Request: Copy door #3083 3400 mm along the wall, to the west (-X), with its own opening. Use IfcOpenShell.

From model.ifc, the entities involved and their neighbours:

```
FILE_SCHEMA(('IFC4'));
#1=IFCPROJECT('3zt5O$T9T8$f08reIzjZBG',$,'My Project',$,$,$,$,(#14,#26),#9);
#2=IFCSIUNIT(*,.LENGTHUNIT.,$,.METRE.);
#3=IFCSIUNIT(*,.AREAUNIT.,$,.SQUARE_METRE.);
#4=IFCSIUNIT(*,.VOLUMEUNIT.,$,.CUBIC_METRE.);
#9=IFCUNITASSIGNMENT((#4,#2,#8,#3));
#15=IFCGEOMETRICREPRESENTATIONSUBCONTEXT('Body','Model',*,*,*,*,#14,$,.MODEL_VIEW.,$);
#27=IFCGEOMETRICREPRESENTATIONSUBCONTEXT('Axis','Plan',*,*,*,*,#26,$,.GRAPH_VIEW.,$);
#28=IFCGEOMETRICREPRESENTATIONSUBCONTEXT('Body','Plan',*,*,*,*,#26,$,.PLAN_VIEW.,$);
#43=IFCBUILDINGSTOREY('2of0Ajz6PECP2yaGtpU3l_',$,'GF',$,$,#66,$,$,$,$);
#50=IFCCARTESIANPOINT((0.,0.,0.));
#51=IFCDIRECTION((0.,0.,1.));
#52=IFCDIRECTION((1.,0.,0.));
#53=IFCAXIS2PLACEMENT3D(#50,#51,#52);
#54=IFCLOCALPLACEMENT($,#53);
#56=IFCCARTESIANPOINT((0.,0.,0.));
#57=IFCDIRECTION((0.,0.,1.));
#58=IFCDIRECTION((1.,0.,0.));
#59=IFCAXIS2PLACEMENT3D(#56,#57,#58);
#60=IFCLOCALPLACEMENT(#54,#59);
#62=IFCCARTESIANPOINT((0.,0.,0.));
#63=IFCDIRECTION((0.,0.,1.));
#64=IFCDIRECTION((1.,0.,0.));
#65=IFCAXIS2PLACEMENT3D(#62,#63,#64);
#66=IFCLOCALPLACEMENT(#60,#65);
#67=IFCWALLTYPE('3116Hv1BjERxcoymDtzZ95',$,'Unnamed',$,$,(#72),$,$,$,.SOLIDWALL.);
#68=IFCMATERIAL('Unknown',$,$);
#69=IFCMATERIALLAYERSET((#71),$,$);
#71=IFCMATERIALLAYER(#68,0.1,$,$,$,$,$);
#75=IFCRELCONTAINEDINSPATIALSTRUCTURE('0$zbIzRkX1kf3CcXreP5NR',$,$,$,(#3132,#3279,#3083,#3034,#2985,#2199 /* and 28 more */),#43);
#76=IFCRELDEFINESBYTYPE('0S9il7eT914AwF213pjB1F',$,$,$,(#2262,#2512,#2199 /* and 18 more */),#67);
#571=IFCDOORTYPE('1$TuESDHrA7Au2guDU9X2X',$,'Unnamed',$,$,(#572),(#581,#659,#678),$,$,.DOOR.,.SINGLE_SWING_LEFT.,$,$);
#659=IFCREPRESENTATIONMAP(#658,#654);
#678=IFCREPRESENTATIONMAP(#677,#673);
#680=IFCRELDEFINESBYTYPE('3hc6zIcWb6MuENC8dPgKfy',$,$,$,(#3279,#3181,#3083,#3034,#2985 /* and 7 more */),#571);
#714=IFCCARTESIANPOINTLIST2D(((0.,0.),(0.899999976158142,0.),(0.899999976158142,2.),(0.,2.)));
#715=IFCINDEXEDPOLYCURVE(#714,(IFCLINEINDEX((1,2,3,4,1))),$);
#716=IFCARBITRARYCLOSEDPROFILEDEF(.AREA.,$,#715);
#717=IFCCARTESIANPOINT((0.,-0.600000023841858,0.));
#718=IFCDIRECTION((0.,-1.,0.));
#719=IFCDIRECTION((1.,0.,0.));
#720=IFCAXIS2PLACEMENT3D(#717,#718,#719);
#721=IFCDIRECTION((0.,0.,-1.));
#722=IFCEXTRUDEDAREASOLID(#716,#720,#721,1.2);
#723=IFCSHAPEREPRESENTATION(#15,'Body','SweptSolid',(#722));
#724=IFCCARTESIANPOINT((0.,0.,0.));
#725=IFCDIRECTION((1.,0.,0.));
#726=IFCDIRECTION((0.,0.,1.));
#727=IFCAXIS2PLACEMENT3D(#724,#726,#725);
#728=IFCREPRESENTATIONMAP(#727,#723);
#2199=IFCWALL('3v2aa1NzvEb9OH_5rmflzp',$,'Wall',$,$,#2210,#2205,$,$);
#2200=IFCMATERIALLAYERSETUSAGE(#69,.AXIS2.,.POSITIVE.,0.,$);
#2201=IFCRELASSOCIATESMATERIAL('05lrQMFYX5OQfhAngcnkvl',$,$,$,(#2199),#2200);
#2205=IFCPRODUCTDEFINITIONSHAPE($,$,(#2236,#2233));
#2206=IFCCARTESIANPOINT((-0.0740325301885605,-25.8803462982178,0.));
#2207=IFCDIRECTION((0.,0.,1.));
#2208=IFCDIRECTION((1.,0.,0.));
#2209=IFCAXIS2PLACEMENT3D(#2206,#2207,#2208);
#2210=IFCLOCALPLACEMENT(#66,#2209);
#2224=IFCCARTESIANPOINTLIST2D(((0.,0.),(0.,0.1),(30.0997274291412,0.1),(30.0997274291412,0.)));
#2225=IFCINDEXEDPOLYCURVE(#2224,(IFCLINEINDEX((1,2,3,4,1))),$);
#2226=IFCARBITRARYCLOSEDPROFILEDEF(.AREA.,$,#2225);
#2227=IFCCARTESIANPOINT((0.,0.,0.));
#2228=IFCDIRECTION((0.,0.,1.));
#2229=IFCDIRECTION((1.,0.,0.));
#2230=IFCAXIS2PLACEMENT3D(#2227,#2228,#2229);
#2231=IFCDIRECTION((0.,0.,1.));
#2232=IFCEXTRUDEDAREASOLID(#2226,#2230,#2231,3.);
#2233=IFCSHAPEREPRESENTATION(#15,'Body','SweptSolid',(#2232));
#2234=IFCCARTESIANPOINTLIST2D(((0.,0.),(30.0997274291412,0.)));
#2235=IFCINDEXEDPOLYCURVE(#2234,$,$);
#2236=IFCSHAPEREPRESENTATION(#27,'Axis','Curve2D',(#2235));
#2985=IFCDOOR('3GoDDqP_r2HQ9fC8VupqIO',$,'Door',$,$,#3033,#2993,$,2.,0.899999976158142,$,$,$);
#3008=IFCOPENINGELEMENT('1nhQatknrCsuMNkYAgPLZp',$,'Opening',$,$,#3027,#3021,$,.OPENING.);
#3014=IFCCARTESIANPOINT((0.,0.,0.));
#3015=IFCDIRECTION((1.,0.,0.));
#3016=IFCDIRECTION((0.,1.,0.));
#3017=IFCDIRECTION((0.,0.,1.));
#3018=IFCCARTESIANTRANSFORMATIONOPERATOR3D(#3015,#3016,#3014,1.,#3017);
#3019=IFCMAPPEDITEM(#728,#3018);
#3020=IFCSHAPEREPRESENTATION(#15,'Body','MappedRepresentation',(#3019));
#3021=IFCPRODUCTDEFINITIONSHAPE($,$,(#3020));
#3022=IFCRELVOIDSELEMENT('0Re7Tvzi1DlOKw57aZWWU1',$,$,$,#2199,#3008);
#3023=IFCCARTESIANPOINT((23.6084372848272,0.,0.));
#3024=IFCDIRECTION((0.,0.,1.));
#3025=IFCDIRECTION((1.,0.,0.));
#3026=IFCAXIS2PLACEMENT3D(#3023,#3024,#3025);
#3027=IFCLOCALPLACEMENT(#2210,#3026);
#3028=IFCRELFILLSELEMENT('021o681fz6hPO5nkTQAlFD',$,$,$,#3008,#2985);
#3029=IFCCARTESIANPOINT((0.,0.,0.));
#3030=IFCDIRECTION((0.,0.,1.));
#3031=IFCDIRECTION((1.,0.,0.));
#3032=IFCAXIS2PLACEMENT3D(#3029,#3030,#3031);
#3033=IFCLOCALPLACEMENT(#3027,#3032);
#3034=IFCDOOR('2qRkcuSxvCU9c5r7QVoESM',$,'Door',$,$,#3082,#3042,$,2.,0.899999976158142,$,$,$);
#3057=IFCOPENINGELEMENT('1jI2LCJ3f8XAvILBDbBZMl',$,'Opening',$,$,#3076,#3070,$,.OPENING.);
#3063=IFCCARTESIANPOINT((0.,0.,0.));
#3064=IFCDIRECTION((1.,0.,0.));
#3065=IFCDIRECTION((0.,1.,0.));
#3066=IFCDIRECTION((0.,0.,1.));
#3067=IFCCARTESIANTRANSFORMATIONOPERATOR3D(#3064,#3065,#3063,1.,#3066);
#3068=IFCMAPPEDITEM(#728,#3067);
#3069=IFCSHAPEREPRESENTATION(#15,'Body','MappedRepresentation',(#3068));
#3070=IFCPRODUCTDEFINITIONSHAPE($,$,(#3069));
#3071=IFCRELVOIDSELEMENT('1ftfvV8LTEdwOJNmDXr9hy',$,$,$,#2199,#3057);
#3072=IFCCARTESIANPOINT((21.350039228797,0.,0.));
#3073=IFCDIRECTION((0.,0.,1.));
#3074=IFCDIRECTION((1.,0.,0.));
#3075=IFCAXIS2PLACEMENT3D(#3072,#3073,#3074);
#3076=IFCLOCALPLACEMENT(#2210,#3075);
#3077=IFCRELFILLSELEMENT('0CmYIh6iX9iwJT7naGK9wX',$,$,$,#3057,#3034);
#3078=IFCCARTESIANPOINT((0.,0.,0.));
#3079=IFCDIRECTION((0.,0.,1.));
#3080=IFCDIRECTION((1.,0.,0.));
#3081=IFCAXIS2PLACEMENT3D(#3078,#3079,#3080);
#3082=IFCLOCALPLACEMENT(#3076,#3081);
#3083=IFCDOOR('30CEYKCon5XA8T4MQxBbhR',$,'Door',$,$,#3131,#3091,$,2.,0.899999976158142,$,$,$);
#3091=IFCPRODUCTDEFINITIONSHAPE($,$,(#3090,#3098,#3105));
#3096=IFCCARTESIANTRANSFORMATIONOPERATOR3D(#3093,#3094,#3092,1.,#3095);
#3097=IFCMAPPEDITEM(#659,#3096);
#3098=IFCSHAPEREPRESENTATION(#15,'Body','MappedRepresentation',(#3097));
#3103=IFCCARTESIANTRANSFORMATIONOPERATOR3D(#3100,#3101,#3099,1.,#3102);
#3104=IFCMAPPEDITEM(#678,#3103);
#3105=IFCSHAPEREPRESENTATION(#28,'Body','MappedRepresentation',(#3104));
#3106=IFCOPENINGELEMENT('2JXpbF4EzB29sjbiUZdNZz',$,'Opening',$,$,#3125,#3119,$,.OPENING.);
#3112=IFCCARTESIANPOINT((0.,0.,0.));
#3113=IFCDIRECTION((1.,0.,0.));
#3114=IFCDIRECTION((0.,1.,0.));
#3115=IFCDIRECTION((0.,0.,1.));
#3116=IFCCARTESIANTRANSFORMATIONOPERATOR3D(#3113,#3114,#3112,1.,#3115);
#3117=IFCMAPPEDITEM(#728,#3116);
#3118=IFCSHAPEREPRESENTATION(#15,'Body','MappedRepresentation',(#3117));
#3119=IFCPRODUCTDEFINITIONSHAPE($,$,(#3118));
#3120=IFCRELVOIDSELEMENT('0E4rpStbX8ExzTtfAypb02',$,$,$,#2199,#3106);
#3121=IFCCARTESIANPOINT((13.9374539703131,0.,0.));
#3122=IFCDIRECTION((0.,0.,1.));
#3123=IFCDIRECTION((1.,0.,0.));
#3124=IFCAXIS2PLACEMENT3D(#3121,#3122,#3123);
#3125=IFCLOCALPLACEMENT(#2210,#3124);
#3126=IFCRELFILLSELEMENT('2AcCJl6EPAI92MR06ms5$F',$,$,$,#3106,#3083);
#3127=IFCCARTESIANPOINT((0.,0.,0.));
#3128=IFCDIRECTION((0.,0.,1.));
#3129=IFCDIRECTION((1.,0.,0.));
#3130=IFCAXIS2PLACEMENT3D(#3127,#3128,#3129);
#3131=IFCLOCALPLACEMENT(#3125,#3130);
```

```python
import ifcopenshell
import ifcopenshell.api.feature
import ifcopenshell.api.geometry
import ifcopenshell.api.root
import ifcopenshell.geom
import ifcopenshell.util.element
import ifcopenshell.util.placement
import ifcopenshell.util.shape
import ifcopenshell.util.unit

model = ifcopenshell.open("model.ifc")
unit_scale = ifcopenshell.util.unit.calculate_unit_scale(model)
settings = ifcopenshell.geom.settings()


def volume(element):
    """Net volume in cubic metres, openings subtracted."""
    shape = ifcopenshell.geom.create_shape(settings, element)
    return ifcopenshell.util.shape.get_volume(shape.geometry)


door = model.by_guid("30CEYKCon5XA8T4MQxBbhR")
opening = door.FillsVoids[0].RelatingOpeningElement
wall = opening.VoidsElements[0].RelatingBuildingElement
before = volume(wall)
shift = ifcopenshell.util.placement.get_local_placement(wall.ObjectPlacement)[:3, 0] * -3.4 / unit_scale

# copy_class copies the void relationship, type, container and properties, but no geometry.
new_opening = ifcopenshell.api.root.copy_class(model, product=opening)
new_opening.Representation = ifcopenshell.util.element.copy_deep(
    model, opening.Representation, exclude=["IfcGeometricRepresentationContext", "IfcRepresentationMap"]
)
new_door = ifcopenshell.api.root.copy_class(model, product=door)
new_door.Representation = ifcopenshell.util.element.copy_deep(
    model, door.Representation, exclude=["IfcGeometricRepresentationContext", "IfcRepresentationMap"]
)
ifcopenshell.api.feature.add_filling(model, opening=new_opening, element=new_door)

for old, new in ((opening, new_opening), (door, new_door)):
    matrix = ifcopenshell.util.placement.get_local_placement(old.ObjectPlacement)
    matrix[:3, 3] += shift
    ifcopenshell.api.geometry.edit_object_placement(model, product=new, matrix=matrix, is_si=False)

after = volume(wall)

print(f"wall volume {before:.3f} -> {after:.3f} m3")

model.write("model-out.ifc")
```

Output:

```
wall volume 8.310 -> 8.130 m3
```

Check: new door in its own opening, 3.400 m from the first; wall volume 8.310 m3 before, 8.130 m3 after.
